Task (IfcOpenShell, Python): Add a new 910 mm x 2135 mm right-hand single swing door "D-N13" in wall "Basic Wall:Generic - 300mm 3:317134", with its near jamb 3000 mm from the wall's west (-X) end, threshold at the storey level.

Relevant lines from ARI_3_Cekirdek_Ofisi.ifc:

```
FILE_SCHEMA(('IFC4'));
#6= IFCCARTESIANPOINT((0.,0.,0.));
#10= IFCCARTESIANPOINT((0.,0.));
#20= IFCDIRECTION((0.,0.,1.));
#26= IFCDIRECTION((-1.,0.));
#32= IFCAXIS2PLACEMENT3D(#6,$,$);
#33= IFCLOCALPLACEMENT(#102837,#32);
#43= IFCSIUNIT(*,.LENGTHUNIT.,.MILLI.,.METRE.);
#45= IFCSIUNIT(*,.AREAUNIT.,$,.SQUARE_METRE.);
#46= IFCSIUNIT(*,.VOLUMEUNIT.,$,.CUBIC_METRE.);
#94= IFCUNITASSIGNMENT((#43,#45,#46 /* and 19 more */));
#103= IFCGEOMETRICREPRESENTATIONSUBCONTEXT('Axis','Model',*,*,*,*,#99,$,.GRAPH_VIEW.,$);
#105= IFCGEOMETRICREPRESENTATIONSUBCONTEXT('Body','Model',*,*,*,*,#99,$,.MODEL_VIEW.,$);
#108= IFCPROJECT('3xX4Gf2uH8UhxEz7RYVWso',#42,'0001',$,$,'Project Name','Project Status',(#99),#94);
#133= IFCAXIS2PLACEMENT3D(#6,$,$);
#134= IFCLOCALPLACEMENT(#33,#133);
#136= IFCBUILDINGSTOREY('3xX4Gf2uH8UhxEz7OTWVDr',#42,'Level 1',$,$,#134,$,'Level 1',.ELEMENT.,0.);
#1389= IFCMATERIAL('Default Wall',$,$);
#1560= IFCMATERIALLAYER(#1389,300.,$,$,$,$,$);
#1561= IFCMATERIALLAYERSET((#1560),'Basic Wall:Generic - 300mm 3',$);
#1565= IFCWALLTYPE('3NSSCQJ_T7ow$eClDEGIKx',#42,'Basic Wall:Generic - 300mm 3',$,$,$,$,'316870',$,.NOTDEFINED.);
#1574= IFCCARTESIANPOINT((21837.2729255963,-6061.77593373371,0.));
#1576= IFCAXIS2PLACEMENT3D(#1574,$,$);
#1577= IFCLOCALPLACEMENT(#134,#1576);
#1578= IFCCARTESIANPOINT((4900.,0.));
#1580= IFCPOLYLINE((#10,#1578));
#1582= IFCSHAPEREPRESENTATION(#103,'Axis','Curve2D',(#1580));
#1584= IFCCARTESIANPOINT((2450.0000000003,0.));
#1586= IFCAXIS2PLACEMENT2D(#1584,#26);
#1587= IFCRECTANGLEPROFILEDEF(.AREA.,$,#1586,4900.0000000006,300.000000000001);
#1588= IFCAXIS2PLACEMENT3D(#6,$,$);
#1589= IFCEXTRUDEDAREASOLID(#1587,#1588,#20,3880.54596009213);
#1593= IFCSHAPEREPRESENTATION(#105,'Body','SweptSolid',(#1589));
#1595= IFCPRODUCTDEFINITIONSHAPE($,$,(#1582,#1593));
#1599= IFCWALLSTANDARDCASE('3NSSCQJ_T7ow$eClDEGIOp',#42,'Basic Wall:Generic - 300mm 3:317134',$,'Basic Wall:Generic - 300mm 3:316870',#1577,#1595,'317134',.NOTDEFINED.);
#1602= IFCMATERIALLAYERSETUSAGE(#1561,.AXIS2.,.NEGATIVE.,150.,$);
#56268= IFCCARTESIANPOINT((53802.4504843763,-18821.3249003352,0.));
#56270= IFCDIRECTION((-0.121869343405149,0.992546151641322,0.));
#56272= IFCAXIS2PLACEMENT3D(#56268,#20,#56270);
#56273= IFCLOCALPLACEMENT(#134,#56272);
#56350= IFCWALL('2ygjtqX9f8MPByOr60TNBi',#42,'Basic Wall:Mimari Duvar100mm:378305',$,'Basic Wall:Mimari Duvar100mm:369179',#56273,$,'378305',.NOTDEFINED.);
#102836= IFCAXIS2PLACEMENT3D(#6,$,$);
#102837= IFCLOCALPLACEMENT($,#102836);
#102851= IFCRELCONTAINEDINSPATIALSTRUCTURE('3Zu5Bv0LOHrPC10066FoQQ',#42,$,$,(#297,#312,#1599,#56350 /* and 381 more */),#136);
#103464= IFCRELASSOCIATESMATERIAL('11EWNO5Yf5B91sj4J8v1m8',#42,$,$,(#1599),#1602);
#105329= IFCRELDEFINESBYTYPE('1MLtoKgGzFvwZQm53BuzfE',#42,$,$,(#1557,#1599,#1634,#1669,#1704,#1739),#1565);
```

```python
import numpy as np
import ifcopenshell
import ifcopenshell.api.feature
import ifcopenshell.api.geometry
import ifcopenshell.api.root
import ifcopenshell.api.spatial
import ifcopenshell.geom
import ifcopenshell.util.element
import ifcopenshell.util.placement
import ifcopenshell.util.representation
import ifcopenshell.util.shape
import ifcopenshell.util.unit

model = ifcopenshell.open("ARI_3_Cekirdek_Ofisi.ifc")
unit_scale = ifcopenshell.util.unit.calculate_unit_scale(model)
settings = ifcopenshell.geom.settings()


def volume(element):
    """Net volume in cubic metres, openings subtracted."""
    shape = ifcopenshell.geom.create_shape(settings, element)
    return ifcopenshell.util.shape.get_volume(shape.geometry)


wall = model.by_guid("3NSSCQJ_T7ow$eClDEGIOp")
storey = ifcopenshell.util.element.get_container(wall, ifc_class="IfcBuildingStorey")
context = ifcopenshell.util.representation.get_context(model, "Model", "Body", "MODEL_VIEW")
before = volume(wall)

width, height, from_end, sill = 0.91, 2.135, 3, 0.0  # metres

# The wall runs along its own X axis, and the end named is its -X end.
wall_shape = ifcopenshell.geom.create_shape(settings, wall)
x, y, z = ifcopenshell.util.shape.get_vertices(wall_shape.geometry).T
start = x.min() + from_end
face, thickness = float(y.min()), float(y.max() - y.min())
wall_matrix = ifcopenshell.util.placement.get_local_placement(wall.ObjectPlacement)
level = ifcopenshell.util.placement.get_local_placement(storey.ObjectPlacement)[2, 3]


def in_wall(x, y):
    """Placement at x, y metres in the wall's axes, at sill height."""
    matrix = wall_matrix.copy()
    matrix[:, 3] = wall_matrix @ np.array([x / unit_scale, y / unit_scale, 0.0, 1.0])
    matrix[2, 3] = level + sill / unit_scale
    return matrix


# Opening: a box that overshoots both wall faces by 50 mm.
opening = ifcopenshell.api.root.create_entity(model, ifc_class="IfcOpeningElement", predefined_type="OPENING")
box = ifcopenshell.api.geometry.add_wall_representation(
    model, context=context, length=width, height=height, thickness=thickness + 0.1
)
ifcopenshell.api.geometry.assign_representation(model, product=opening, representation=box)
ifcopenshell.api.geometry.edit_object_placement(model, product=opening, matrix=in_wall(start, face - 0.05), is_si=False)
ifcopenshell.api.feature.add_feature(model, feature=opening, element=wall)

door = ifcopenshell.api.root.create_entity(model, ifc_class="IfcDoor", name="D-N13", predefined_type="DOOR")
door.OverallWidth, door.OverallHeight = width / unit_scale, height / unit_scale
door.OperationType = "SINGLE_SWING_RIGHT"
body = ifcopenshell.api.geometry.add_door_representation(
    model,
    context=context,
    overall_width=door.OverallWidth,
    overall_height=door.OverallHeight,
    operation_type="SINGLE_SWING_RIGHT",
    lining_properties={"LiningDepth": thickness / unit_scale, "ThresholdDepth": thickness / unit_scale},
)
ifcopenshell.api.geometry.assign_representation(model, product=door, representation=body)
ifcopenshell.api.spatial.assign_container(model, products=[door], relating_structure=storey)
ifcopenshell.api.feature.add_filling(model, opening=opening, element=door)

# The lining spans the wall, so the door starts at the wall face.
ifcopenshell.api.geometry.edit_object_placement(model, product=door, matrix=in_wall(start, face), is_si=False)

after = volume(wall)

print(f"wall volume {before:.3f} -> {after:.3f} m3")

model.write("ARI_3_Cekirdek_Ofisi_v2.ifc")
```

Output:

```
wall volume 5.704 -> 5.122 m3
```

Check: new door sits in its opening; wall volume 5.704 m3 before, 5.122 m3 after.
